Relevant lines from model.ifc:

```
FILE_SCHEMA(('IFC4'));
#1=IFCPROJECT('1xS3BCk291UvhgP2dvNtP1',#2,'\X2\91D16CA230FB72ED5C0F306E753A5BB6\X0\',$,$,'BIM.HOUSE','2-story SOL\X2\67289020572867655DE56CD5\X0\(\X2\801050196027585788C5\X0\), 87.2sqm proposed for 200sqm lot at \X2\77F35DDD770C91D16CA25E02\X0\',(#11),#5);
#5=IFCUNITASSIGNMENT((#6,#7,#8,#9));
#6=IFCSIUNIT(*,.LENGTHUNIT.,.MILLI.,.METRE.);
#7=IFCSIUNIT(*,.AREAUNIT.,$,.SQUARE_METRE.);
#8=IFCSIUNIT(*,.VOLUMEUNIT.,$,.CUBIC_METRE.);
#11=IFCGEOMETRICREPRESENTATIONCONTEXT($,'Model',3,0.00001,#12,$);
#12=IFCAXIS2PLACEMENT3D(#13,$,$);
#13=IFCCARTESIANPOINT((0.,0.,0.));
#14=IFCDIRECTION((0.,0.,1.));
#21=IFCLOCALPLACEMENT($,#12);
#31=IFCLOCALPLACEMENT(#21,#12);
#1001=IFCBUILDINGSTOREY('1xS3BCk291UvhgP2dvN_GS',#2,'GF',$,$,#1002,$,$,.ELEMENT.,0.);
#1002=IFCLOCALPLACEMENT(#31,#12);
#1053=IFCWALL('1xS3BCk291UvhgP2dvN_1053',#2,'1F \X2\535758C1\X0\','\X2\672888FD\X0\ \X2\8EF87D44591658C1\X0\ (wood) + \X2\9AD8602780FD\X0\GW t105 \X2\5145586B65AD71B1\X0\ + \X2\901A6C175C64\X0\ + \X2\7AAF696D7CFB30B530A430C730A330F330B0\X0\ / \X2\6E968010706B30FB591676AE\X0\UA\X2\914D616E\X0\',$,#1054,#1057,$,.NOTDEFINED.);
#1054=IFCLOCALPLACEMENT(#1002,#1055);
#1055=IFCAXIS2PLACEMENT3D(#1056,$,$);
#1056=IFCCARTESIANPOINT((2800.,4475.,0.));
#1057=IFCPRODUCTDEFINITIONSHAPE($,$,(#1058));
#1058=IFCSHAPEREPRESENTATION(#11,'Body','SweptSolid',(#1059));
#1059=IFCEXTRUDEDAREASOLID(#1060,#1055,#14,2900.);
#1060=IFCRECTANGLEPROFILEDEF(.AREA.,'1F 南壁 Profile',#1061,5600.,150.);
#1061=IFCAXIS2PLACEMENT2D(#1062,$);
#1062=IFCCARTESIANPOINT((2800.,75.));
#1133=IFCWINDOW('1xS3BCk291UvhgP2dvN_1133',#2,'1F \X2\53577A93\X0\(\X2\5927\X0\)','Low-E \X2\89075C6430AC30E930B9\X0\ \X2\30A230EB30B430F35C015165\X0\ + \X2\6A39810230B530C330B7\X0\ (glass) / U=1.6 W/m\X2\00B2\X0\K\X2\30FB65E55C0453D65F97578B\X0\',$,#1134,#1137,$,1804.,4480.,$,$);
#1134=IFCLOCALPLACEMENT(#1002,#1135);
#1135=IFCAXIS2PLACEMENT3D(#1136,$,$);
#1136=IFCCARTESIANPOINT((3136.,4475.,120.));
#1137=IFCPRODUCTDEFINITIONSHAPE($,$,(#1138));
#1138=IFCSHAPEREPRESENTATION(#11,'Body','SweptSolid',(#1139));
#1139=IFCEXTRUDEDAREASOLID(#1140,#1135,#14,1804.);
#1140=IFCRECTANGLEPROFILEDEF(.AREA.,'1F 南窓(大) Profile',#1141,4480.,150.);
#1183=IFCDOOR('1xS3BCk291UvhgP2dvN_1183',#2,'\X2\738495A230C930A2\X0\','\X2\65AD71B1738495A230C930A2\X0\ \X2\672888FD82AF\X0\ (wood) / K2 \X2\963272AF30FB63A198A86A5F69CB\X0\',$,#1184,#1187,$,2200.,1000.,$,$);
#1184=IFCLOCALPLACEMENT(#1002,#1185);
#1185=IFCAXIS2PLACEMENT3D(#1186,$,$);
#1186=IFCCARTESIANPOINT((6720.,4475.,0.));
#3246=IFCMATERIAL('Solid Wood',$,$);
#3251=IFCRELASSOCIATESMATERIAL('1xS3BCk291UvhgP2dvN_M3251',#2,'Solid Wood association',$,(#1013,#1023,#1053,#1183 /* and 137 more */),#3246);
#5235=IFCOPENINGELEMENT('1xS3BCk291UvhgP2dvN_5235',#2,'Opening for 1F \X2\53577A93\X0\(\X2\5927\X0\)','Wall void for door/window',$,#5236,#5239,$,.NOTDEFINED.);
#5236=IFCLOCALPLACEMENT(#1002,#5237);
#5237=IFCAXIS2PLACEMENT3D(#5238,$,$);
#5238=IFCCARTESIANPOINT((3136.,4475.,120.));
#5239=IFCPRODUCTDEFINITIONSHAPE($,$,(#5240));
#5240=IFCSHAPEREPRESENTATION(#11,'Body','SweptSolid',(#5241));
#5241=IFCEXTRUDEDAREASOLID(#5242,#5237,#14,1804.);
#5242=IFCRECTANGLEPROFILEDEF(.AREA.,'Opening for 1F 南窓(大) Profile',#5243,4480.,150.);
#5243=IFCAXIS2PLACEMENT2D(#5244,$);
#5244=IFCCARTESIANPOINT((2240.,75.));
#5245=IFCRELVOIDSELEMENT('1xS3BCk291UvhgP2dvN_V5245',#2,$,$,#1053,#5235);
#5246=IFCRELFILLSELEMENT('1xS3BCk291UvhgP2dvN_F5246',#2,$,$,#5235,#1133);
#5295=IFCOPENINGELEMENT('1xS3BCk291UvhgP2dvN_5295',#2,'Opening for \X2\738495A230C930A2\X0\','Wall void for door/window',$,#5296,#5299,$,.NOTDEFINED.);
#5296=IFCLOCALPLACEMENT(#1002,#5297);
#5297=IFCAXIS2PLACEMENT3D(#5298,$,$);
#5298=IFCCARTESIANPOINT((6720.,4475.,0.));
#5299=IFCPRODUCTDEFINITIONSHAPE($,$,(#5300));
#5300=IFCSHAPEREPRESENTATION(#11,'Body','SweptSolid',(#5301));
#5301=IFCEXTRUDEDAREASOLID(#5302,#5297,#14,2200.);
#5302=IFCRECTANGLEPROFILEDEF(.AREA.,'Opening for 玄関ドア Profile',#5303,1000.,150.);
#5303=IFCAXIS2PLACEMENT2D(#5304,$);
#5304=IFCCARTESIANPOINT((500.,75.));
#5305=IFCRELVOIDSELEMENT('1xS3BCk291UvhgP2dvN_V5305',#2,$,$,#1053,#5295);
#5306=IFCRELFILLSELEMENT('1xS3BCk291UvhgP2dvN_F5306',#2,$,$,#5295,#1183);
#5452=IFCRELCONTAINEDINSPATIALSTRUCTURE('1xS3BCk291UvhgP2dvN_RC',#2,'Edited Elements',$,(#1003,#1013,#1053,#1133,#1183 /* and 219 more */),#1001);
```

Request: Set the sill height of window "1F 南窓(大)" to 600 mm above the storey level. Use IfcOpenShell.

```python
import numpy as np
import ifcopenshell
import ifcopenshell.api.geometry
import ifcopenshell.geom
import ifcopenshell.util.element
import ifcopenshell.util.placement
import ifcopenshell.util.shape
import ifcopenshell.util.unit

model = ifcopenshell.open("model.ifc")
unit_scale = ifcopenshell.util.unit.calculate_unit_scale(model)

window = model.by_guid("1xS3BCk291UvhgP2dvN_1133")
opening = window.FillsVoids[0].RelatingOpeningElement
storey = ifcopenshell.util.element.get_container(window, ifc_class="IfcBuildingStorey")
level = ifcopenshell.util.placement.get_local_placement(storey.ObjectPlacement)[2, 3]

# The opening's origin need not be at the sill, so measure its lowest point.
shape = ifcopenshell.geom.create_shape(ifcopenshell.geom.settings(), opening)
bottom = ifcopenshell.util.shape.get_shape_bottom_elevation(shape, shape.geometry) / unit_scale
dz = level + 0.6 / unit_scale - bottom

shift = np.array([0.0, 0.0, dz])
# The window is not placed relative to its opening, so move both.
for product in (opening, window):
    matrix = ifcopenshell.util.placement.get_local_placement(product.ObjectPlacement)
    matrix[:3, 3] += shift
    ifcopenshell.api.geometry.edit_object_placement(model, product=product, matrix=matrix, is_si=False)

print(f"moved by {dz * unit_scale:+.3f} m")

model.write("model_rev.ifc")
```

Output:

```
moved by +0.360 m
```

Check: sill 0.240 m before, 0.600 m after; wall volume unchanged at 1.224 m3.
